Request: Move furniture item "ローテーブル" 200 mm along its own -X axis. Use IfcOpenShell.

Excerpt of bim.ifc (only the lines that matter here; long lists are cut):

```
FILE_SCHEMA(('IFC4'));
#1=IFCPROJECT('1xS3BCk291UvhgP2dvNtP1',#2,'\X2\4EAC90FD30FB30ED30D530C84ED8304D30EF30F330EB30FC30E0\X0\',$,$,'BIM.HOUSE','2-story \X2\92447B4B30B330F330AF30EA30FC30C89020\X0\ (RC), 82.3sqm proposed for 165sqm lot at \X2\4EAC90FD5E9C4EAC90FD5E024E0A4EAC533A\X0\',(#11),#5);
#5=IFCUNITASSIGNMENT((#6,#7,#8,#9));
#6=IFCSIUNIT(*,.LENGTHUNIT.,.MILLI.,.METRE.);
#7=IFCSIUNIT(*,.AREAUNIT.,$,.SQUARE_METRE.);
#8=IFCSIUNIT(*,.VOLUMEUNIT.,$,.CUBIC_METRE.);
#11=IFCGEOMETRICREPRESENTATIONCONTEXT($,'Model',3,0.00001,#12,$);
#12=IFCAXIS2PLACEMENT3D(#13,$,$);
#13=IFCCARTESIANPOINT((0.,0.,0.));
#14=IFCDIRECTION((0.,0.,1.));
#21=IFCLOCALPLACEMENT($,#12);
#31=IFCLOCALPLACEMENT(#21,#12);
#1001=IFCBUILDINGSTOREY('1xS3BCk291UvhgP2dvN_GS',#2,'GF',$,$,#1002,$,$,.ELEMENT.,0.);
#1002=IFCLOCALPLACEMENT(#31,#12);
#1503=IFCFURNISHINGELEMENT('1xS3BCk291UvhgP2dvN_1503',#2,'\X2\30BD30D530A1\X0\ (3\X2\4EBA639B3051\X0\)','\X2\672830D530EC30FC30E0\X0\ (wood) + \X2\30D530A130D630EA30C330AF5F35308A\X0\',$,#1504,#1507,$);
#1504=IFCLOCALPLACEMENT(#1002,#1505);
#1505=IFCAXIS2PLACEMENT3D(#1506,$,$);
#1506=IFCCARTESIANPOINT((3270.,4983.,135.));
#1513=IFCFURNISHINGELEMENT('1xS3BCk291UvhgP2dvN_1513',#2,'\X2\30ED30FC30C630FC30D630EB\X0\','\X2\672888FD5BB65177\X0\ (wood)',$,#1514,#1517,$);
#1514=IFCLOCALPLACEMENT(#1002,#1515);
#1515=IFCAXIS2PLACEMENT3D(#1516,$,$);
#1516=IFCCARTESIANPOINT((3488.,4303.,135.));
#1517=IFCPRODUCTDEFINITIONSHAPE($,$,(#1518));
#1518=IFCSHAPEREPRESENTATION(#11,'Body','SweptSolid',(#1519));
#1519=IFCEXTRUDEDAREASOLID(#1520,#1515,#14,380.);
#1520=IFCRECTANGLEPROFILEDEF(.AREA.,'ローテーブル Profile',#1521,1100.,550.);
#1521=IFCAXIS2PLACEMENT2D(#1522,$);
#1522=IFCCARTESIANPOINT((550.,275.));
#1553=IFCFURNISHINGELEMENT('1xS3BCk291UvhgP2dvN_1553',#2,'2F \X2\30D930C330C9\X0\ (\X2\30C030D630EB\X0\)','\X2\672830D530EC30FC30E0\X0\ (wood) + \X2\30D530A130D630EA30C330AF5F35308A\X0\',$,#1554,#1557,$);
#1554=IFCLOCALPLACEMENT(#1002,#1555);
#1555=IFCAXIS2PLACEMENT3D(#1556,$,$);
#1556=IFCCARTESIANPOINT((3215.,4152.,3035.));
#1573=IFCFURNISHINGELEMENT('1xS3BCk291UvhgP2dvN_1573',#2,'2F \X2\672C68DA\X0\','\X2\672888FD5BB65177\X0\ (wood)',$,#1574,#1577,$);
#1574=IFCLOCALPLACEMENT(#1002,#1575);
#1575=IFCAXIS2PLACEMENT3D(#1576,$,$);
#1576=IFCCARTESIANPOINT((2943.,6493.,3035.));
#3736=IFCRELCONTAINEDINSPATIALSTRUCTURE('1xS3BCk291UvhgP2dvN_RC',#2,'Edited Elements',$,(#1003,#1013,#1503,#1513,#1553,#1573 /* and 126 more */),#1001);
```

```python
import ifcopenshell
import ifcopenshell.api.geometry
import ifcopenshell.util.placement
import ifcopenshell.util.unit

model = ifcopenshell.open("bim.ifc")
unit_scale = ifcopenshell.util.unit.calculate_unit_scale(model)

item = model.by_guid("1xS3BCk291UvhgP2dvN_1513")
matrix = ifcopenshell.util.placement.get_local_placement(item.ObjectPlacement)
matrix[:3, 3] -= matrix[:3, 0] * 0.2 / unit_scale
ifcopenshell.api.geometry.edit_object_placement(model, product=item, matrix=matrix, is_si=False)

print(ifcopenshell.util.placement.get_local_placement(item.ObjectPlacement).round(3) + 0.0)

model.write("bim_v2.ifc")
```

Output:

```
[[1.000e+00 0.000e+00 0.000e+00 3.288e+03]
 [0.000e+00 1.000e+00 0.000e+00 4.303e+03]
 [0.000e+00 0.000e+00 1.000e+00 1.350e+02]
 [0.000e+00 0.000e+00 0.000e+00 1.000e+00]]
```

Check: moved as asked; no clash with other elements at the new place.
